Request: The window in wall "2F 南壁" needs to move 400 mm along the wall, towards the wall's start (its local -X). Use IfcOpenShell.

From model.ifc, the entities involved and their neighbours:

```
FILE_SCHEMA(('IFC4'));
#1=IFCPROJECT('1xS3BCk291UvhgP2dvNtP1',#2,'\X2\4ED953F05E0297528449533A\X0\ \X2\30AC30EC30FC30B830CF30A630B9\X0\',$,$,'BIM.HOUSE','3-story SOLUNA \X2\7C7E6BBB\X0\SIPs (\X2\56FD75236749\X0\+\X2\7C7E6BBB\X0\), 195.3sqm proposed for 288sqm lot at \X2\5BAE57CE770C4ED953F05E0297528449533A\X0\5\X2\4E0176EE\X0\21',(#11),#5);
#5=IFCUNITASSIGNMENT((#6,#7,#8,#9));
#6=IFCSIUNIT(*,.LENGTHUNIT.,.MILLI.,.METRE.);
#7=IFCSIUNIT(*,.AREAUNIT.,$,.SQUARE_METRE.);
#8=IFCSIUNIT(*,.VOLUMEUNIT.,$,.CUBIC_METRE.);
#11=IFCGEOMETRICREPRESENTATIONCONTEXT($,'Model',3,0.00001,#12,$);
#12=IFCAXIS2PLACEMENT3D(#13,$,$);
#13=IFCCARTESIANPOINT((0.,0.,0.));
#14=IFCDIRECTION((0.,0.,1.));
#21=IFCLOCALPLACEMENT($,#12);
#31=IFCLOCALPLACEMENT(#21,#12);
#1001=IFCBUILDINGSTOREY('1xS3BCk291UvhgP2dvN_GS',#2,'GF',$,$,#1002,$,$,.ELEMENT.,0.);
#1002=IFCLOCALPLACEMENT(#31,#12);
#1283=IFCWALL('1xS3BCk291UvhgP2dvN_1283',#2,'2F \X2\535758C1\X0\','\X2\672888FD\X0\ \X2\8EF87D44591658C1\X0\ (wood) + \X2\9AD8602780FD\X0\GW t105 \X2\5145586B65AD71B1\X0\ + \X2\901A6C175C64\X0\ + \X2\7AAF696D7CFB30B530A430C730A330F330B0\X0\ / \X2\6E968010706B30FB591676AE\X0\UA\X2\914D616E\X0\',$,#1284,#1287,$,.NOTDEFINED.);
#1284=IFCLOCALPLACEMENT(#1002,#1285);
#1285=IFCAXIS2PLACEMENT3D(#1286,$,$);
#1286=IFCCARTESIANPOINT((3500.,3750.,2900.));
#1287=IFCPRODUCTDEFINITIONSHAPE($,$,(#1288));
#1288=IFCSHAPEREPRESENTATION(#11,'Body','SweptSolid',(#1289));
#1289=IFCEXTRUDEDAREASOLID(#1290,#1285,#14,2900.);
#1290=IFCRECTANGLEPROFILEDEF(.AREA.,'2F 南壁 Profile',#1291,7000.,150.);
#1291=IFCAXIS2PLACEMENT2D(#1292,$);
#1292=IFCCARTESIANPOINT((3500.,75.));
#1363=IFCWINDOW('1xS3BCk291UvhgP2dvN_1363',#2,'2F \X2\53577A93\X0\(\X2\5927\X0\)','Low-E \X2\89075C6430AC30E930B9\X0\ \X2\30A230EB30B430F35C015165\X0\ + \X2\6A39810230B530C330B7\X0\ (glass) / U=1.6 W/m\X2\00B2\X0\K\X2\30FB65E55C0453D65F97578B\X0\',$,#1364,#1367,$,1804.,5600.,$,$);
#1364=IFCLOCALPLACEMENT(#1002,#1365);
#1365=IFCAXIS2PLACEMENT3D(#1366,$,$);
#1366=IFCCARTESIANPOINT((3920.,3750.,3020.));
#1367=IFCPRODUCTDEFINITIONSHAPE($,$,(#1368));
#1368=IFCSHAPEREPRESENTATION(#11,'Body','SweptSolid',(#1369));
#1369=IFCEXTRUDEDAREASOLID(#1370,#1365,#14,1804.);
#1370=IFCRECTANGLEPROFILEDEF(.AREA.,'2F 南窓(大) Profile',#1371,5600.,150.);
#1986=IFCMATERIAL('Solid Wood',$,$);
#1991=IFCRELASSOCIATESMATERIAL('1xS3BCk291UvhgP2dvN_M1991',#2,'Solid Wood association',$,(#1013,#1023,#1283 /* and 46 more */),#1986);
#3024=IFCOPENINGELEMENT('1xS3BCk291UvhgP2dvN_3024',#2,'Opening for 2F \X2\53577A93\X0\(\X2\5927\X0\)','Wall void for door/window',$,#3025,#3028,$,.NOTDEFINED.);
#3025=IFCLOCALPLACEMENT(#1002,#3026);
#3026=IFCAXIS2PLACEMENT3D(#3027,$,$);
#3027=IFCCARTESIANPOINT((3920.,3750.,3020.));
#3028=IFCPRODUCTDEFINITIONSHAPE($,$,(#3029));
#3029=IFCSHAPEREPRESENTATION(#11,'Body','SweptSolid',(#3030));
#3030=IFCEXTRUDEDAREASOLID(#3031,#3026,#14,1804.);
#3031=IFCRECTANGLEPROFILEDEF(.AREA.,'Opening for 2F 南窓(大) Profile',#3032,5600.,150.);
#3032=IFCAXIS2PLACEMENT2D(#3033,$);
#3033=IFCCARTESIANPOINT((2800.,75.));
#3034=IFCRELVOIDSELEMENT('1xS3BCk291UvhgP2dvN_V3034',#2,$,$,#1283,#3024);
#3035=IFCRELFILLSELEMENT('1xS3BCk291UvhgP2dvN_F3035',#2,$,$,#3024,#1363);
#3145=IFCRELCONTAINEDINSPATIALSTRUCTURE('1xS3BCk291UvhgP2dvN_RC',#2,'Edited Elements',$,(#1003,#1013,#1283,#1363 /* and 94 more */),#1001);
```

```python
import ifcopenshell
import ifcopenshell.api.geometry
import ifcopenshell.util.placement

model = ifcopenshell.open("model.ifc")

window = model.by_guid("1xS3BCk291UvhgP2dvN_1363")
opening = window.FillsVoids[0].RelatingOpeningElement
wall = opening.VoidsElements[0].RelatingBuildingElement

wall_matrix = ifcopenshell.util.placement.get_local_placement(wall.ObjectPlacement)
shift = wall_matrix[:3, 0] * -400.0
before = ifcopenshell.util.placement.get_local_placement(window.ObjectPlacement)[:3, 3].copy()

# The window is not placed relative to its opening, so move both.
for product in (opening, window):
    matrix = ifcopenshell.util.placement.get_local_placement(product.ObjectPlacement)
    matrix[:3, 3] += shift
    ifcopenshell.api.geometry.edit_object_placement(model, product=product, matrix=matrix, is_si=False)

after = ifcopenshell.util.placement.get_local_placement(window.ObjectPlacement)[:3, 3]
print("window moved by", (after - before).round(3) + 0.0)

model.write("model_updated.ifc")
```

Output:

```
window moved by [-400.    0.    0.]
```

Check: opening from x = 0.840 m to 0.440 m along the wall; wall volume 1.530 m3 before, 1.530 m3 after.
